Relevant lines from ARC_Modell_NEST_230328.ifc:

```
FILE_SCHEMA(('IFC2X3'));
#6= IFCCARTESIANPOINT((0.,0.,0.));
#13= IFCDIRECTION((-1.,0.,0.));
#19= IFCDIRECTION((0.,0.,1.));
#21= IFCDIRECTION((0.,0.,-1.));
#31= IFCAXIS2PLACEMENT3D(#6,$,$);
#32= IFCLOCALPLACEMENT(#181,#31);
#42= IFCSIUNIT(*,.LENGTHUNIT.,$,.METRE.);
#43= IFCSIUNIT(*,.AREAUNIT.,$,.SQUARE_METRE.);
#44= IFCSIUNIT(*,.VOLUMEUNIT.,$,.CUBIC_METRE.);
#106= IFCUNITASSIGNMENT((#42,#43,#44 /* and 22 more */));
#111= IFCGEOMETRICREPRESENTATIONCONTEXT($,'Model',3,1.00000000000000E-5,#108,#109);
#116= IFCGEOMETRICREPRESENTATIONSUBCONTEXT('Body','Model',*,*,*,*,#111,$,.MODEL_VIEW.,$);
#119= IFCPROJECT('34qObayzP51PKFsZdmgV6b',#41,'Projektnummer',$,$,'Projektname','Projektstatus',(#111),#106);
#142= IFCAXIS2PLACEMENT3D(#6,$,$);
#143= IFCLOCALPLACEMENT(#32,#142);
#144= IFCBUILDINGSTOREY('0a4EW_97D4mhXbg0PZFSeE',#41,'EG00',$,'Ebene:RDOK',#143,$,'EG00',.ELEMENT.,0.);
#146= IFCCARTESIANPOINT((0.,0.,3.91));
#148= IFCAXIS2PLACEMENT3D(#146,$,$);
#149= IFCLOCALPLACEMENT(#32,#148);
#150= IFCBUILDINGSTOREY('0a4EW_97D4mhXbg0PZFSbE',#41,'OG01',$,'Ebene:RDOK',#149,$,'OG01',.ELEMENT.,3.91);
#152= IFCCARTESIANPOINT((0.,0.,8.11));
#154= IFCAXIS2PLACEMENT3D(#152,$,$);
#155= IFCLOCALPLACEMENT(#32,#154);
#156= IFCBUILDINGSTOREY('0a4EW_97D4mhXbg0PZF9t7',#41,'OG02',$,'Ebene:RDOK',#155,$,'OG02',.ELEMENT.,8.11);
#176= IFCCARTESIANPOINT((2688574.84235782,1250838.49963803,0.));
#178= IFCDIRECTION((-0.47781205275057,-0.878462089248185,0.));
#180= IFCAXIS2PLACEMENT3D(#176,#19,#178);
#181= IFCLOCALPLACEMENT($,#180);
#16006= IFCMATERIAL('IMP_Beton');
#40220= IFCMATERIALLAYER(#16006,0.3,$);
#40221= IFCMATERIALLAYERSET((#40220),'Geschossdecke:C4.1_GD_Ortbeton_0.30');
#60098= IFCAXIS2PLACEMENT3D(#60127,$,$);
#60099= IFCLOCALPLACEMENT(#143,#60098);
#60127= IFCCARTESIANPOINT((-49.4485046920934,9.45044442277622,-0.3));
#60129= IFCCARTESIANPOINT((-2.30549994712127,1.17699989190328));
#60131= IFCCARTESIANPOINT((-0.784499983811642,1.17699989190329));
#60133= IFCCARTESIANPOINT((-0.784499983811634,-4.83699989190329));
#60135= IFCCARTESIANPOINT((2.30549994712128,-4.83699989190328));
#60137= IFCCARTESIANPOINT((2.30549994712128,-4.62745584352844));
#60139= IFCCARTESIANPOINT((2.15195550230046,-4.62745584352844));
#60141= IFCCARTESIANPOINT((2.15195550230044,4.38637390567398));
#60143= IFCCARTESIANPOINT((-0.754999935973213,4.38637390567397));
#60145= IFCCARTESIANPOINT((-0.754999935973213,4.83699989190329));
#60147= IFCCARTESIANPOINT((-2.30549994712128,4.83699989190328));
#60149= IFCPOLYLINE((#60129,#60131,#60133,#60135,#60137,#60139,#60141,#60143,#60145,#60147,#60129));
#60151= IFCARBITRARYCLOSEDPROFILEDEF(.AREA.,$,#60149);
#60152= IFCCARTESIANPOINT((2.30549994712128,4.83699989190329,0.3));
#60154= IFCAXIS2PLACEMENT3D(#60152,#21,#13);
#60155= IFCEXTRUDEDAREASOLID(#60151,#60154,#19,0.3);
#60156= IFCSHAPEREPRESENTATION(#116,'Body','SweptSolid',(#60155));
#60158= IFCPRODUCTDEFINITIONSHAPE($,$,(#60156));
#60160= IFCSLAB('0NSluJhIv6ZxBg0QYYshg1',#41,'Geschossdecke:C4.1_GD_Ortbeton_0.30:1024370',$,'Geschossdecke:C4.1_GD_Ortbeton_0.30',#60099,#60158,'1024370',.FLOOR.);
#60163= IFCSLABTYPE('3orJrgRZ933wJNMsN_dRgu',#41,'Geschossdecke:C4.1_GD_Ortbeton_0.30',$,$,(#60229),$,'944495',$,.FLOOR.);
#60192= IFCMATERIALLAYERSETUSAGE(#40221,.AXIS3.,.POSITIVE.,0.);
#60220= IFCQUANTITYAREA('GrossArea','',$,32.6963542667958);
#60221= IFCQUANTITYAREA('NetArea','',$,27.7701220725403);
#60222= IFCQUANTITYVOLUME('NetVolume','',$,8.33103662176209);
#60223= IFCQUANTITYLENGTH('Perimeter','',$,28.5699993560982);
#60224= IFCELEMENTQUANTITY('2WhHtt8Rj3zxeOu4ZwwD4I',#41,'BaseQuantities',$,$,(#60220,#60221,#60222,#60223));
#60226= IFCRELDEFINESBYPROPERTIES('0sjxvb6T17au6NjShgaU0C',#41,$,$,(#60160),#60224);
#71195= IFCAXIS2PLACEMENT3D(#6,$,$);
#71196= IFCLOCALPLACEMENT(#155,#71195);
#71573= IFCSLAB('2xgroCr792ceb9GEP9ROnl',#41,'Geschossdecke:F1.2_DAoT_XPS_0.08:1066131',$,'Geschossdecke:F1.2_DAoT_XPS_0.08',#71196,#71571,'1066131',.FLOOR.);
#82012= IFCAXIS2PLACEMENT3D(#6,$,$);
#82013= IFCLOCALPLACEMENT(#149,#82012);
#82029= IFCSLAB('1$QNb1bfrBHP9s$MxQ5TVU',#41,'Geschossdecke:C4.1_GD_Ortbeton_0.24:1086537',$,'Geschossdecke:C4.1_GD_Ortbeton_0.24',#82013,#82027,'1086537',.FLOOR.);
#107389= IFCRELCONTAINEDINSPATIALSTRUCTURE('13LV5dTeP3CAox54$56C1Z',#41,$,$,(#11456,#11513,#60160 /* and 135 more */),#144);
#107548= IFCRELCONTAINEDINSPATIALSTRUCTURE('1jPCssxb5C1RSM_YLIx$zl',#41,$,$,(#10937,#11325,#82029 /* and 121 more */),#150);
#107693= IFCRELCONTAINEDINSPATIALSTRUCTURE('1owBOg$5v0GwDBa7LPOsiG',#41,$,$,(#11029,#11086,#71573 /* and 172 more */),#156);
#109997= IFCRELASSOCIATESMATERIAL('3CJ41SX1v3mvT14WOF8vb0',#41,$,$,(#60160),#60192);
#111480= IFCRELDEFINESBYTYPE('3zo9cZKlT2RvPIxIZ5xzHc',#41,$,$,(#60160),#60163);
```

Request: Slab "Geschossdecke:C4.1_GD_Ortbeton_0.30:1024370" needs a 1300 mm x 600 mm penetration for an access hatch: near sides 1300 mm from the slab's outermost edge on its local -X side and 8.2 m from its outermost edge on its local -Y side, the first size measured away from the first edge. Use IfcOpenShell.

```python
import numpy as np
import ifcopenshell
import ifcopenshell.api.feature
import ifcopenshell.api.geometry
import ifcopenshell.api.pset
import ifcopenshell.api.root
import ifcopenshell.geom
import ifcopenshell.util.element
import ifcopenshell.util.placement
import ifcopenshell.util.representation
import ifcopenshell.util.shape
import ifcopenshell.util.unit

model = ifcopenshell.open("ARC_Modell_NEST_230328.ifc")
unit_scale = ifcopenshell.util.unit.calculate_unit_scale(model)
area_scale = ifcopenshell.util.unit.calculate_unit_scale(model, "AREAUNIT")
volume_scale = ifcopenshell.util.unit.calculate_unit_scale(model, "VOLUMEUNIT")
settings = ifcopenshell.geom.settings()


def volume(element):
    """Net volume in cubic metres, openings subtracted."""
    shape = ifcopenshell.geom.create_shape(settings, element)
    return ifcopenshell.util.shape.get_volume(shape.geometry)


slab = model.by_guid("0NSluJhIv6ZxBg0QYYshg1")
before = volume(slab)

# Extent in the slab's own axes, in metres. The edges named are its -X and -Y sides.
slab_shape = ifcopenshell.geom.create_shape(settings, slab)
vertices = ifcopenshell.util.shape.get_vertices(slab_shape.geometry)
x_min, y_min, bottom = vertices.min(axis=0)
top = vertices[:, 2].max()

opening = ifcopenshell.api.root.create_entity(model, ifc_class="IfcOpeningElement", name="Access hatch opening")
context = ifcopenshell.util.representation.get_context(model, "Model", "Body", "MODEL_VIEW")
width, depth = 1.3, 0.6
outline = [(0.0, 0.0), (width, 0.0), (width, depth), (0.0, depth), (0.0, 0.0)]
# Overshoot both faces by 50 mm so the cut is clean.
shape = ifcopenshell.api.geometry.add_slab_representation(
    model, context=context, depth=top - bottom + 0.1, polyline=outline
)
ifcopenshell.api.geometry.assign_representation(model, product=opening, representation=shape)

matrix = ifcopenshell.util.placement.get_local_placement(slab.ObjectPlacement)
matrix[:, 3] = matrix @ np.append(np.array([x_min + 1.3, y_min + 8.2, bottom - 0.05]) / unit_scale, 1.0)
ifcopenshell.api.geometry.edit_object_placement(model, product=opening, matrix=matrix, is_si=False)
ifcopenshell.api.feature.add_feature(model, feature=opening, element=slab)

after = volume(slab)

# Update the slab's stored quantities.
qto = model.by_id(ifcopenshell.util.element.get_pset(slab, "BaseQuantities", should_inherit=False)["id"])
ifcopenshell.api.pset.edit_qto(model, qto=qto, properties={
    "NetArea": after / (top - bottom) / area_scale,
    "NetVolume": after / volume_scale,
})

print(f"slab volume {before:.3f} -> {after:.3f} m3")

model.write("ARC_Modell_NEST_230328_v2.ifc")
```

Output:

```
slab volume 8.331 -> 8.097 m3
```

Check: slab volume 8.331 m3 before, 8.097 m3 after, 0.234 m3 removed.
